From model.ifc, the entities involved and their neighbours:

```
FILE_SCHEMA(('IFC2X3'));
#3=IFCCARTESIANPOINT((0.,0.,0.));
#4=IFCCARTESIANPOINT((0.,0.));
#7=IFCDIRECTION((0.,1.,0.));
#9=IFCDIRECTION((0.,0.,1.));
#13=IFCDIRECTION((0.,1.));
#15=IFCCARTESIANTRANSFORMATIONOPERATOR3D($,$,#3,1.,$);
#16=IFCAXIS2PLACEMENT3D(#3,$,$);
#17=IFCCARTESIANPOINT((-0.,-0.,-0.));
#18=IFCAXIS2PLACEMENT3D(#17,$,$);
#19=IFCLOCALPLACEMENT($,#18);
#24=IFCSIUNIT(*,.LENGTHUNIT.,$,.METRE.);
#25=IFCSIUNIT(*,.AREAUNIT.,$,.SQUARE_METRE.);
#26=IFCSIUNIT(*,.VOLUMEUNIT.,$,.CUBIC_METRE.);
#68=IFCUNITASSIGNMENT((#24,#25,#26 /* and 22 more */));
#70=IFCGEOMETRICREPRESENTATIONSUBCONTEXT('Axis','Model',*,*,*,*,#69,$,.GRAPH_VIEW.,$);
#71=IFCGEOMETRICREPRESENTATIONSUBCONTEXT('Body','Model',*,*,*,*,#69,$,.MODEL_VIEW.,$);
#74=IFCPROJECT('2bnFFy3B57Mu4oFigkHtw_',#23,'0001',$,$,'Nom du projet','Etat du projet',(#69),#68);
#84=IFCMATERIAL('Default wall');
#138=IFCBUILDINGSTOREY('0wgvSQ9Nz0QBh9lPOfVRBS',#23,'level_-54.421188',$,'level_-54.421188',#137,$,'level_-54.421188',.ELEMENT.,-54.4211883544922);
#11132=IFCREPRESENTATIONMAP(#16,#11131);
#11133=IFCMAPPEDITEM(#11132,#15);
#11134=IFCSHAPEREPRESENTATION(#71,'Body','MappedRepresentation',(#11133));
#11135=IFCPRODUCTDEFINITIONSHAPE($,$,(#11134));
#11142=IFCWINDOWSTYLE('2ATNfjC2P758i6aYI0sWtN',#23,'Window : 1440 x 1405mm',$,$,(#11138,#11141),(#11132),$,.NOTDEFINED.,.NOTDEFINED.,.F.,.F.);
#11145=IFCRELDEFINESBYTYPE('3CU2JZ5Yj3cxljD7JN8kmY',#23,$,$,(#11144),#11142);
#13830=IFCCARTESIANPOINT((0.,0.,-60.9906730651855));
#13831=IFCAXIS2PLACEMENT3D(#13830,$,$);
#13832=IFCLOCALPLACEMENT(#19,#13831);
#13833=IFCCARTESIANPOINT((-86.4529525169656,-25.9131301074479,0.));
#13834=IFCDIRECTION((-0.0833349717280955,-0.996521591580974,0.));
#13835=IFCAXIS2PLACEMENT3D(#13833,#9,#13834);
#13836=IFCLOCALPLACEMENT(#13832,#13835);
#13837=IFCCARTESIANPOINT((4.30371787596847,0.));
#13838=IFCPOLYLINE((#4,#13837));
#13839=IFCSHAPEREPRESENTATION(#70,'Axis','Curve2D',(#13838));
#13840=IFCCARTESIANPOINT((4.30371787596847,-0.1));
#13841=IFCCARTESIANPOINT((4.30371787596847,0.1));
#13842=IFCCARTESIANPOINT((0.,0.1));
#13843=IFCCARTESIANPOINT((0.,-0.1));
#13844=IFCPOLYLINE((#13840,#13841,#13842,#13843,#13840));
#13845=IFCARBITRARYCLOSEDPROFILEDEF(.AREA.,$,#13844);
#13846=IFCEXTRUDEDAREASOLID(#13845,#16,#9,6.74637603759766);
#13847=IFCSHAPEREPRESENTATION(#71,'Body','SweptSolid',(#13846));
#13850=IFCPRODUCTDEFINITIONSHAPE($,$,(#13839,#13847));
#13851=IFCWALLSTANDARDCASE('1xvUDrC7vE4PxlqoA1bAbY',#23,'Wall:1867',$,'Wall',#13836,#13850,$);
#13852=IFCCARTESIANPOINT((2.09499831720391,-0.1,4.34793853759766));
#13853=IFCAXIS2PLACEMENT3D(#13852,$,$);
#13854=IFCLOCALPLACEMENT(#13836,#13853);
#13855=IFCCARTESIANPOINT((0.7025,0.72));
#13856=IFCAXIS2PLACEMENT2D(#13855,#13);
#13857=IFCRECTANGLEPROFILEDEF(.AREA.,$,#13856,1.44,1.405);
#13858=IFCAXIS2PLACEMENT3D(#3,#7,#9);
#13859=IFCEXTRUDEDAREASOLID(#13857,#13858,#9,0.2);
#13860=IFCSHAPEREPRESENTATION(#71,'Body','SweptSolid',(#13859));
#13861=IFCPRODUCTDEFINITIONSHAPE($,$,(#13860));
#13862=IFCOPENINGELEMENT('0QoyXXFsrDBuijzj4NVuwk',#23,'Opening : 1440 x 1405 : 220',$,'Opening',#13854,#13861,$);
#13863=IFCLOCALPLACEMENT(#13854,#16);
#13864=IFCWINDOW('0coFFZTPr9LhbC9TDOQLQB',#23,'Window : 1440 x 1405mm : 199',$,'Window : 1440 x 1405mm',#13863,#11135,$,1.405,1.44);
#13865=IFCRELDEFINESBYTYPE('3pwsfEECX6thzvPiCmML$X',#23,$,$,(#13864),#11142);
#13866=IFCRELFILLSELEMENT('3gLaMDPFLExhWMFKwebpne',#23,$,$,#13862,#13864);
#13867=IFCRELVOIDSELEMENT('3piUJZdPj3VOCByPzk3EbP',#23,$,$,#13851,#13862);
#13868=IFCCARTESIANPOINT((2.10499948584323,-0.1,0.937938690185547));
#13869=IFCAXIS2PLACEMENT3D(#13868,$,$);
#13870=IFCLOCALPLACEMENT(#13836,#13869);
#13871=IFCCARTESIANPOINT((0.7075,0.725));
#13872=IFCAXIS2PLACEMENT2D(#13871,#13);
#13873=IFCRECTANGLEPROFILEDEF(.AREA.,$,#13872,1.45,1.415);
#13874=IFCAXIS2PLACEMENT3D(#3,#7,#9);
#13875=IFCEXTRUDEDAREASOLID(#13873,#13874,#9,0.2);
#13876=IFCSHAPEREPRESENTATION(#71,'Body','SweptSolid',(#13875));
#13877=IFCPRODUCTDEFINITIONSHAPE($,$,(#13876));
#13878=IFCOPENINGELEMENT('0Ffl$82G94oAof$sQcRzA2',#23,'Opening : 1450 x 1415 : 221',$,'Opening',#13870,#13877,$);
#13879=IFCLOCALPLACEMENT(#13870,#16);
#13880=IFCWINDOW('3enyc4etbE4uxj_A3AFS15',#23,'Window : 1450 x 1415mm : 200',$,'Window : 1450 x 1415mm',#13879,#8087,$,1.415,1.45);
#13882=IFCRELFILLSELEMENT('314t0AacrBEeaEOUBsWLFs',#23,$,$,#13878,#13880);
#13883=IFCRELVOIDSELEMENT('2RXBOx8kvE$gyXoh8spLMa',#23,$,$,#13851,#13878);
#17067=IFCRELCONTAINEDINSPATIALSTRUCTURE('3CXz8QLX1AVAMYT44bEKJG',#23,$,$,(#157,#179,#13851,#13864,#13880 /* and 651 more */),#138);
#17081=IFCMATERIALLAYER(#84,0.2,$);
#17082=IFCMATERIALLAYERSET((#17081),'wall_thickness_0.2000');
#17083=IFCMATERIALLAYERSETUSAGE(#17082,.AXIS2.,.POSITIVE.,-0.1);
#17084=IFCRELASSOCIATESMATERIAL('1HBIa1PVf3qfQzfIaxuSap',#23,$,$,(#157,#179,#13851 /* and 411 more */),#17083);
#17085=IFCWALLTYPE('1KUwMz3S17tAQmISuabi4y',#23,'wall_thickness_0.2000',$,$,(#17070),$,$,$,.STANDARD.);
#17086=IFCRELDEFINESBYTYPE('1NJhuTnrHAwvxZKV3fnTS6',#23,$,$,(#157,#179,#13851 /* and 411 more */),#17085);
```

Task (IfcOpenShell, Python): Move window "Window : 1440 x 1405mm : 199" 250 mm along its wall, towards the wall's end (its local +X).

```python
import ifcopenshell
import ifcopenshell.api.geometry
import ifcopenshell.util.placement
import ifcopenshell.util.unit

model = ifcopenshell.open("model.ifc")
unit_scale = ifcopenshell.util.unit.calculate_unit_scale(model)

window = model.by_guid("0coFFZTPr9LhbC9TDOQLQB")
opening = window.FillsVoids[0].RelatingOpeningElement
wall = opening.VoidsElements[0].RelatingBuildingElement

wall_matrix = ifcopenshell.util.placement.get_local_placement(wall.ObjectPlacement)
shift = wall_matrix[:3, 0] * 0.25 / unit_scale
before = ifcopenshell.util.placement.get_local_placement(window.ObjectPlacement)[:3, 3].copy()

# The window is placed relative to its opening, so it follows when the opening moves.
matrix = ifcopenshell.util.placement.get_local_placement(opening.ObjectPlacement)
matrix[:3, 3] += shift
ifcopenshell.api.geometry.edit_object_placement(
    model, product=opening, matrix=matrix, is_si=False, should_transform_children=True
)

after = ifcopenshell.util.placement.get_local_placement(window.ObjectPlacement)[:3, 3]
print("window moved by", (after - before).round(3) + 0.0)

model.write("model_v2.ifc")
```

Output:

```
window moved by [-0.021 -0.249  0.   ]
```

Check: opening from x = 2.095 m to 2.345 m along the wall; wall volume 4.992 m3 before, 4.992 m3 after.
